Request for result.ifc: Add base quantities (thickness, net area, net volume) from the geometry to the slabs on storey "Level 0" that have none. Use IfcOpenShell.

First a look at what the model holds.

```python
import ifcopenshell
import ifcopenshell.util.element
import ifcopenshell.util.unit

model = ifcopenshell.open("result.ifc")
print(model.schema)
for unit_type in ("LENGTHUNIT", "AREAUNIT", "VOLUMEUNIT"):
    print(unit_type, ifcopenshell.util.unit.calculate_unit_scale(model, unit_type))
storey = next(s for s in model.by_type("IfcBuildingStorey") if s.Name == "Level 0")
slabs = [e for e in ifcopenshell.util.element.get_decomposition(storey) if e.is_a("IfcSlab")]
for e in sorted(slabs, key=lambda e: e.id()):
    print(e.id(), e.is_a(), e.Name, list(ifcopenshell.util.element.get_psets(e, qtos_only=True)), sep=" | ")
```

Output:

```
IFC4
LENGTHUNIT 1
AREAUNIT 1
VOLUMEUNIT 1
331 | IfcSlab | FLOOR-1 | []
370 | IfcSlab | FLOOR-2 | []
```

```python
import ifcopenshell
import ifcopenshell.api.pset
import ifcopenshell.geom
import ifcopenshell.util.element
import ifcopenshell.util.shape
import ifcopenshell.util.unit

model = ifcopenshell.open("result.ifc")
unit_scale = ifcopenshell.util.unit.calculate_unit_scale(model)
area_scale = ifcopenshell.util.unit.calculate_unit_scale(model, "AREAUNIT")
volume_scale = ifcopenshell.util.unit.calculate_unit_scale(model, "VOLUMEUNIT")
settings = ifcopenshell.geom.settings()

storey = next(s for s in model.by_type("IfcBuildingStorey") if s.Name == "Level 0")
slabs = [e for e in ifcopenshell.util.element.get_decomposition(storey) if e.is_a("IfcSlab")]

for e in sorted(slabs, key=lambda e: e.id()):
    if ifcopenshell.util.element.get_psets(e, qtos_only=True, should_inherit=False):
        continue
    # Geometry comes back in metres, in the element's own axes.
    shape = ifcopenshell.geom.create_shape(settings, e)
    values = {
        "Width": ifcopenshell.util.shape.get_z(shape.geometry) / unit_scale,
        "NetArea": ifcopenshell.util.shape.get_footprint_area(shape.geometry) / area_scale,
        "NetVolume": ifcopenshell.util.shape.get_volume(shape.geometry) / volume_scale,
    }
    qto = ifcopenshell.api.pset.add_qto(model, product=e, name="Qto_SlabBaseQuantities")
    ifcopenshell.api.pset.edit_qto(model, qto=qto, properties=values)
    print(e.id(), {k: round(v, 3) for k, v in values.items()})

model.write("result_rev.ifc")
```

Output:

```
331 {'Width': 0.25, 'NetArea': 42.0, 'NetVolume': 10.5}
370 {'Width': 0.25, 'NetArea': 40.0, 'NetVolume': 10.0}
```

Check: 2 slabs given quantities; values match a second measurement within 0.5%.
